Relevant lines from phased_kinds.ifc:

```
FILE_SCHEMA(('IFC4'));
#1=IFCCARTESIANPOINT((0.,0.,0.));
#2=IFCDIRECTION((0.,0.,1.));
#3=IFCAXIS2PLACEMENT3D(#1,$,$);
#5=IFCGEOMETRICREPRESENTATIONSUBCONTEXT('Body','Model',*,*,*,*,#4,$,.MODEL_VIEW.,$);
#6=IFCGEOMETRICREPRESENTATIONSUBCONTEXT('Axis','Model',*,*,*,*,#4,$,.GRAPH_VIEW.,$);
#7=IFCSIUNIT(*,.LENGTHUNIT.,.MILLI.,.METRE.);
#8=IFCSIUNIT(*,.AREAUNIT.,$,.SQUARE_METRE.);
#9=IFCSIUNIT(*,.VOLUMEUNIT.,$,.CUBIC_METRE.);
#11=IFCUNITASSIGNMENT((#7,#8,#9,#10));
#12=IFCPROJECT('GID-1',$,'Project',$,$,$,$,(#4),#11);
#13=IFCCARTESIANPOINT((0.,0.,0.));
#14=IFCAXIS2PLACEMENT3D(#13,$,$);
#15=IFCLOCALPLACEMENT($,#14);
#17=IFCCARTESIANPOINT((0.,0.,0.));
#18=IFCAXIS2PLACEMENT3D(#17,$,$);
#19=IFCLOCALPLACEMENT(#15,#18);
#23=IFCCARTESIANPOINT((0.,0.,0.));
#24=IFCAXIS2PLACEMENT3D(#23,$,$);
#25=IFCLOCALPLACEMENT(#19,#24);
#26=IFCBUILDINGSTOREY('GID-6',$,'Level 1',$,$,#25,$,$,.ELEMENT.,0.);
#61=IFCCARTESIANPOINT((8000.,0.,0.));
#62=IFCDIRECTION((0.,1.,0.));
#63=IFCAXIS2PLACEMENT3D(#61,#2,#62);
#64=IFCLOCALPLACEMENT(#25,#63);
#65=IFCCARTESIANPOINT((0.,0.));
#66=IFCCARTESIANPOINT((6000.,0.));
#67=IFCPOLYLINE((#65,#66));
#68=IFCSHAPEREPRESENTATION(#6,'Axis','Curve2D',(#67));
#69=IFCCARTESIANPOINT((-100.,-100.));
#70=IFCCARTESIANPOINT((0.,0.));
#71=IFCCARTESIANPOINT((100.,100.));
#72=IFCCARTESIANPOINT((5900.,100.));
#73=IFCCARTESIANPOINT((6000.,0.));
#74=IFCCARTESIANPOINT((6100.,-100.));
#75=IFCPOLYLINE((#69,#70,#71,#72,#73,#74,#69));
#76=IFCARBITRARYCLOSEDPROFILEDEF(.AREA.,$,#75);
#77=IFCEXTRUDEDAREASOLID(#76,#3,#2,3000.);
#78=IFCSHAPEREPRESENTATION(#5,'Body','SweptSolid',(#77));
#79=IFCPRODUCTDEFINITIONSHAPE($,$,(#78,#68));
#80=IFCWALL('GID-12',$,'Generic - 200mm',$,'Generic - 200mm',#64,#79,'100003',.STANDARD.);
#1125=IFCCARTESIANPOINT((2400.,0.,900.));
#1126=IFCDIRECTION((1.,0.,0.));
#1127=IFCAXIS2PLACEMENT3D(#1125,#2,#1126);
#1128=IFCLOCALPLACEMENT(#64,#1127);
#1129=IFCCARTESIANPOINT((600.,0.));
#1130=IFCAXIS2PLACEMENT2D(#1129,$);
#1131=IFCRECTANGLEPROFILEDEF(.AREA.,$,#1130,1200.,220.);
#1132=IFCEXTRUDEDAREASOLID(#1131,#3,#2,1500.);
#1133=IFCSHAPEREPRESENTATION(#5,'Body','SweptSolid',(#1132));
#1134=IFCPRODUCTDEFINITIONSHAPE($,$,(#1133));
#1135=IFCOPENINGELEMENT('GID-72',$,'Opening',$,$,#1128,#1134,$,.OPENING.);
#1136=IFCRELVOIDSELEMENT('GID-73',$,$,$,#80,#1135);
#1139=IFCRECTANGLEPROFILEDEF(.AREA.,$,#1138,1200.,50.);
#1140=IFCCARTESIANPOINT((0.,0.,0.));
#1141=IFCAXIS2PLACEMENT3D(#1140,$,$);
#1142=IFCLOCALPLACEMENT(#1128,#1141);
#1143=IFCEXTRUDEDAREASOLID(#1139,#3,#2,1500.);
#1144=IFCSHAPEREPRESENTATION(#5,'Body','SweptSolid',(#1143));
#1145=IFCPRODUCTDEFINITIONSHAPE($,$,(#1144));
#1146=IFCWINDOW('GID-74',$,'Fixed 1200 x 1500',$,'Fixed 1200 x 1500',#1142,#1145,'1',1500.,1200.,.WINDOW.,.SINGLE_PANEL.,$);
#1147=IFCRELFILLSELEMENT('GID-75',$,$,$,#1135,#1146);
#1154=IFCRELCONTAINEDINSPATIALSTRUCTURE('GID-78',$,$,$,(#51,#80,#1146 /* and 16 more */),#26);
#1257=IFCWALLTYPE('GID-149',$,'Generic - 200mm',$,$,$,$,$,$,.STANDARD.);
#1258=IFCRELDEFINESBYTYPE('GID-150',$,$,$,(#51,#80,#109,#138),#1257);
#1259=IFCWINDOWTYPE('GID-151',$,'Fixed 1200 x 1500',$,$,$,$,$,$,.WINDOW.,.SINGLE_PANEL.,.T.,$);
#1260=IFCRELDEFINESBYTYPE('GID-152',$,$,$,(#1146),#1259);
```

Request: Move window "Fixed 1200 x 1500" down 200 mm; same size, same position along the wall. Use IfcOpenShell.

```python
import numpy as np
import ifcopenshell
import ifcopenshell.api.geometry
import ifcopenshell.util.placement
import ifcopenshell.util.unit

model = ifcopenshell.open("phased_kinds.ifc")
unit_scale = ifcopenshell.util.unit.calculate_unit_scale(model)

window = model.by_guid("GID-74")
opening = window.FillsVoids[0].RelatingOpeningElement
dz = -200.0

shift = np.array([0.0, 0.0, dz])
# The window is placed relative to its opening, so it follows when the opening moves.
matrix = ifcopenshell.util.placement.get_local_placement(opening.ObjectPlacement)
matrix[:3, 3] += shift
ifcopenshell.api.geometry.edit_object_placement(
    model, product=opening, matrix=matrix, is_si=False, should_transform_children=True
)

print(f"moved by {dz * unit_scale:+.3f} m")

model.write("phased_kinds-out.ifc")
```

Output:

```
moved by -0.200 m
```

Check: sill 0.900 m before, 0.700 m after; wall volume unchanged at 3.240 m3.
